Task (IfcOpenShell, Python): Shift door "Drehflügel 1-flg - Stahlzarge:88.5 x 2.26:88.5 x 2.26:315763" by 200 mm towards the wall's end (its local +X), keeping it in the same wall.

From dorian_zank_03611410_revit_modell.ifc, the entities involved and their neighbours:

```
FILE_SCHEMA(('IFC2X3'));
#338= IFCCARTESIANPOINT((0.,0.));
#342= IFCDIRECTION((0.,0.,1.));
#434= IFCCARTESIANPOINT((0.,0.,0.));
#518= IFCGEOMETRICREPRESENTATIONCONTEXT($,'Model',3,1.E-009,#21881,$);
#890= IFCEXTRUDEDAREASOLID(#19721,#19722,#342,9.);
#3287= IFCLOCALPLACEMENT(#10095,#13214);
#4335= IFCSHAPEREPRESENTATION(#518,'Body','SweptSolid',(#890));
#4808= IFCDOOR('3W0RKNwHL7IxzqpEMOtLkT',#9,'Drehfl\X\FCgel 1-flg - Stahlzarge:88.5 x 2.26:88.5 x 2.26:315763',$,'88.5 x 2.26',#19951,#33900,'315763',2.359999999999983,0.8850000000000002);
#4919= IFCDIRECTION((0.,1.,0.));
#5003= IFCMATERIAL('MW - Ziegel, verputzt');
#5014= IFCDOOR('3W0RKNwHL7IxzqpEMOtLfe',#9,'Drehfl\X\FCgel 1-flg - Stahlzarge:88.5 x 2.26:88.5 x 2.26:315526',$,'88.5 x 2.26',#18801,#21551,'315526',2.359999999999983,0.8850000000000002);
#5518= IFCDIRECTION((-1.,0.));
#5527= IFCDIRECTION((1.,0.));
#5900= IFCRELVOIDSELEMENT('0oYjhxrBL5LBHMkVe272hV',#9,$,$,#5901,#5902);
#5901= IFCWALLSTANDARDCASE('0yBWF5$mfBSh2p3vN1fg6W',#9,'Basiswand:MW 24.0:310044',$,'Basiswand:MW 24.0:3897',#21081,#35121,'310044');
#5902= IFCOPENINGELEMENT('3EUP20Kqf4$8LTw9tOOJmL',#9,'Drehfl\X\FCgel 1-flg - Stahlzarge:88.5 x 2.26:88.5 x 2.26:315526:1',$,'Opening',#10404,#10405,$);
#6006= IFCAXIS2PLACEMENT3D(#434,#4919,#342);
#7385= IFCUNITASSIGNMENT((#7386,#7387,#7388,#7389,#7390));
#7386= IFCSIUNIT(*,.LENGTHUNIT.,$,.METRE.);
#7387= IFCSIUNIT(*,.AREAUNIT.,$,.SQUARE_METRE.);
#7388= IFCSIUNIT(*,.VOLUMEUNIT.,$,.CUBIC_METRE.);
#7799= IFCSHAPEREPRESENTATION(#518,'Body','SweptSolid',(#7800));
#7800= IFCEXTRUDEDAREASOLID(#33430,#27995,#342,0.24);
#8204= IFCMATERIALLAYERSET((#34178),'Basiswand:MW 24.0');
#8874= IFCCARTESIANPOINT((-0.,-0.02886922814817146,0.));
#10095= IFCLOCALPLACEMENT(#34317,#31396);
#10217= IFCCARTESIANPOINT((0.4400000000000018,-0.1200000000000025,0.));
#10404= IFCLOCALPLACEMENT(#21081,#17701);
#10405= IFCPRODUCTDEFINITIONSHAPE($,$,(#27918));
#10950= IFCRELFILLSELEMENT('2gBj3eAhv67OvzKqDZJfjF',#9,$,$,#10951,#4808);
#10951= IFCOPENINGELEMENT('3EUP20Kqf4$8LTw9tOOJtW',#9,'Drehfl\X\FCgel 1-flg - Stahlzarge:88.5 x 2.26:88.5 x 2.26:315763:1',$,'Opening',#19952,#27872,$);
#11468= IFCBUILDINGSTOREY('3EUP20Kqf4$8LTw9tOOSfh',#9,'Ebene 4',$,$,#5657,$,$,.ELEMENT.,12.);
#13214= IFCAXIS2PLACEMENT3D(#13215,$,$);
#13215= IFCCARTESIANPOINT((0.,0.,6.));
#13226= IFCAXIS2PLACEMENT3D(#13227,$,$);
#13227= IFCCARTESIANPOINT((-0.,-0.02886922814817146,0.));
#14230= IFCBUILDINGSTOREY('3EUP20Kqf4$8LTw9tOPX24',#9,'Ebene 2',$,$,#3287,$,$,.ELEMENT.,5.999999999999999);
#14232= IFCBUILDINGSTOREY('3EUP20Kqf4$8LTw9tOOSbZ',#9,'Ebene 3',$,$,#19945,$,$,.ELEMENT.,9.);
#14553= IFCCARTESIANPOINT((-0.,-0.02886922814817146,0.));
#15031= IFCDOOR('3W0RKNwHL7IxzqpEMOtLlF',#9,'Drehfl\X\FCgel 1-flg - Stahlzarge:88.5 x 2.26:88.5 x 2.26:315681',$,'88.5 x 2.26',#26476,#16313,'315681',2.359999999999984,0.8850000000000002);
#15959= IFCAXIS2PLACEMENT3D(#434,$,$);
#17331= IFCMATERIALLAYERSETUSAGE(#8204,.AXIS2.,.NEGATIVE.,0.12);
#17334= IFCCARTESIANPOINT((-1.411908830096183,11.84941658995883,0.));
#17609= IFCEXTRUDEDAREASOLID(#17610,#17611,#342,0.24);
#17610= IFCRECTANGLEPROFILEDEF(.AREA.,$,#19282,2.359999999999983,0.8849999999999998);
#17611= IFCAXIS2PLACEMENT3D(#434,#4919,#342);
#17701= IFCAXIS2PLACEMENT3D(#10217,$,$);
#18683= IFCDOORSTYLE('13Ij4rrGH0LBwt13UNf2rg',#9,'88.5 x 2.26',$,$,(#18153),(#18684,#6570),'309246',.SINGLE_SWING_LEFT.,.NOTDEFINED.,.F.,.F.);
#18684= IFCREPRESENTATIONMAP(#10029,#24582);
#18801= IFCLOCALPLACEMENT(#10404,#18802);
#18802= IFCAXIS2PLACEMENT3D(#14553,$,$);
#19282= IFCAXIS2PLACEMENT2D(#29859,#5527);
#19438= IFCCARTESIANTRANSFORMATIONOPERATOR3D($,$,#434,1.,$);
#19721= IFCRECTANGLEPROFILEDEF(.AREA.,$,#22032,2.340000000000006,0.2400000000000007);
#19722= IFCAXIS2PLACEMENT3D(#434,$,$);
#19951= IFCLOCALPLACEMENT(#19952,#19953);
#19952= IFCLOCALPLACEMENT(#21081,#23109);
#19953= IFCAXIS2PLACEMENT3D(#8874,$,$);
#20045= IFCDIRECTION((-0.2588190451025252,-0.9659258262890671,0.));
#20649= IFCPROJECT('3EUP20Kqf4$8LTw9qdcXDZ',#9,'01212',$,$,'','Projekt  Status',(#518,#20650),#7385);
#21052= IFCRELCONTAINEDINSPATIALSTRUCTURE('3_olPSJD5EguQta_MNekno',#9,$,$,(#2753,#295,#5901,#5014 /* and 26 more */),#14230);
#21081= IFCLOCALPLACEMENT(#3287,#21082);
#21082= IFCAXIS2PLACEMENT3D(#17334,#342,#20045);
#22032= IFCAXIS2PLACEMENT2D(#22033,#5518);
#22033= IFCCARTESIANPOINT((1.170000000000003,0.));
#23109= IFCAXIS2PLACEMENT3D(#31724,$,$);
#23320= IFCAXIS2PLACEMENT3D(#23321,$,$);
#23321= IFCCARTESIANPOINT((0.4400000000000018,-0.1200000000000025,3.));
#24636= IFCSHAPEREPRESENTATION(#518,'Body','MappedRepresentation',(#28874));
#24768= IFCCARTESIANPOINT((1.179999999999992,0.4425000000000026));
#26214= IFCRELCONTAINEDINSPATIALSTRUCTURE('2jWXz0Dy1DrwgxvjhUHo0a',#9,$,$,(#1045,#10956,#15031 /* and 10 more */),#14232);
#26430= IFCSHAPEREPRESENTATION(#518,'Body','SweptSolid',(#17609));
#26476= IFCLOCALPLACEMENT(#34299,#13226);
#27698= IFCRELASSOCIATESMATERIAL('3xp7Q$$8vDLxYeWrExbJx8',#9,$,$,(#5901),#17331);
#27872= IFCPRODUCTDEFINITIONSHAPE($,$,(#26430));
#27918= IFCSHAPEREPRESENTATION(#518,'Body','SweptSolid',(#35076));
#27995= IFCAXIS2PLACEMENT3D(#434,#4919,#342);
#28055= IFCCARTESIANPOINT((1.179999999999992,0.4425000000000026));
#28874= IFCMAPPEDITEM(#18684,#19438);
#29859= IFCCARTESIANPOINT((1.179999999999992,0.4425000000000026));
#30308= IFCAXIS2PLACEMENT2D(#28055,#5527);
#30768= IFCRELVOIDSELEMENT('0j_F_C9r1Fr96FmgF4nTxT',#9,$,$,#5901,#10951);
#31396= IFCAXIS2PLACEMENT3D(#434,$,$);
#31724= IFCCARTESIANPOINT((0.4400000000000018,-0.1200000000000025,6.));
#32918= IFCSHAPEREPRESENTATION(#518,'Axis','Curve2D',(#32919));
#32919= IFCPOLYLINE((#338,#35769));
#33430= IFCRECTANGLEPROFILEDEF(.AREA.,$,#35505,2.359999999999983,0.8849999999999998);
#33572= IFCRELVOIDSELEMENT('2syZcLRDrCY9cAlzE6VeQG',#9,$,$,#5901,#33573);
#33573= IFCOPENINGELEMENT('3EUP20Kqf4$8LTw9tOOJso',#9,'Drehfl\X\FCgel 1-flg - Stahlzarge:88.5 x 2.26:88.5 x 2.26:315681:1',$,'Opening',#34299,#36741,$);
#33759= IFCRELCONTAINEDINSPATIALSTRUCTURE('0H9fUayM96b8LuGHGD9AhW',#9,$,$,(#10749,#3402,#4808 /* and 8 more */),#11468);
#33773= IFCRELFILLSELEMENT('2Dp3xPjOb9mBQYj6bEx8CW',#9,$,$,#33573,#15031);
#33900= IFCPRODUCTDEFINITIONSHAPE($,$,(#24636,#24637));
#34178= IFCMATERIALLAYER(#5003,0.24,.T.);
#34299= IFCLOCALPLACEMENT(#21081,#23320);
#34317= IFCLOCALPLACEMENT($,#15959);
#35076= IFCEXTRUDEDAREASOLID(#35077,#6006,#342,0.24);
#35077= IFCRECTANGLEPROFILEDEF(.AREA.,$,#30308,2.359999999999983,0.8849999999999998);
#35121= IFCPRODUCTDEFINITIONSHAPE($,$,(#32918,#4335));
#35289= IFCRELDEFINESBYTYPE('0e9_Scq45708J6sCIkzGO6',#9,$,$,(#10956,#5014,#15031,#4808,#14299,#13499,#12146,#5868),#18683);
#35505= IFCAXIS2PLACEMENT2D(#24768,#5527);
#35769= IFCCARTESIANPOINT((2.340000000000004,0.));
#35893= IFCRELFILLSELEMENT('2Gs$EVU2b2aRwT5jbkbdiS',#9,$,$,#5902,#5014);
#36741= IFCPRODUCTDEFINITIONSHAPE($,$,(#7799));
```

```python
import ifcopenshell
import ifcopenshell.api.geometry
import ifcopenshell.util.placement
import ifcopenshell.util.unit

model = ifcopenshell.open("dorian_zank_03611410_revit_modell.ifc")
unit_scale = ifcopenshell.util.unit.calculate_unit_scale(model)

door = model.by_guid("3W0RKNwHL7IxzqpEMOtLkT")
opening = door.FillsVoids[0].RelatingOpeningElement
wall = opening.VoidsElements[0].RelatingBuildingElement

wall_matrix = ifcopenshell.util.placement.get_local_placement(wall.ObjectPlacement)
shift = wall_matrix[:3, 0] * 0.2 / unit_scale
before = ifcopenshell.util.placement.get_local_placement(door.ObjectPlacement)[:3, 3].copy()

# The door is placed relative to its opening, so it follows when the opening moves.
matrix = ifcopenshell.util.placement.get_local_placement(opening.ObjectPlacement)
matrix[:3, 3] += shift
ifcopenshell.api.geometry.edit_object_placement(
    model, product=opening, matrix=matrix, is_si=False, should_transform_children=True
)

after = ifcopenshell.util.placement.get_local_placement(door.ObjectPlacement)[:3, 3]
print("door moved by", (after - before).round(3) + 0.0)

model.write("dorian_zank_03611410_revit_modell_v2.ifc")
```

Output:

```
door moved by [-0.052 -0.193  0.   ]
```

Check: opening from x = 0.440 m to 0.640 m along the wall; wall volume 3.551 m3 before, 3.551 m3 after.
